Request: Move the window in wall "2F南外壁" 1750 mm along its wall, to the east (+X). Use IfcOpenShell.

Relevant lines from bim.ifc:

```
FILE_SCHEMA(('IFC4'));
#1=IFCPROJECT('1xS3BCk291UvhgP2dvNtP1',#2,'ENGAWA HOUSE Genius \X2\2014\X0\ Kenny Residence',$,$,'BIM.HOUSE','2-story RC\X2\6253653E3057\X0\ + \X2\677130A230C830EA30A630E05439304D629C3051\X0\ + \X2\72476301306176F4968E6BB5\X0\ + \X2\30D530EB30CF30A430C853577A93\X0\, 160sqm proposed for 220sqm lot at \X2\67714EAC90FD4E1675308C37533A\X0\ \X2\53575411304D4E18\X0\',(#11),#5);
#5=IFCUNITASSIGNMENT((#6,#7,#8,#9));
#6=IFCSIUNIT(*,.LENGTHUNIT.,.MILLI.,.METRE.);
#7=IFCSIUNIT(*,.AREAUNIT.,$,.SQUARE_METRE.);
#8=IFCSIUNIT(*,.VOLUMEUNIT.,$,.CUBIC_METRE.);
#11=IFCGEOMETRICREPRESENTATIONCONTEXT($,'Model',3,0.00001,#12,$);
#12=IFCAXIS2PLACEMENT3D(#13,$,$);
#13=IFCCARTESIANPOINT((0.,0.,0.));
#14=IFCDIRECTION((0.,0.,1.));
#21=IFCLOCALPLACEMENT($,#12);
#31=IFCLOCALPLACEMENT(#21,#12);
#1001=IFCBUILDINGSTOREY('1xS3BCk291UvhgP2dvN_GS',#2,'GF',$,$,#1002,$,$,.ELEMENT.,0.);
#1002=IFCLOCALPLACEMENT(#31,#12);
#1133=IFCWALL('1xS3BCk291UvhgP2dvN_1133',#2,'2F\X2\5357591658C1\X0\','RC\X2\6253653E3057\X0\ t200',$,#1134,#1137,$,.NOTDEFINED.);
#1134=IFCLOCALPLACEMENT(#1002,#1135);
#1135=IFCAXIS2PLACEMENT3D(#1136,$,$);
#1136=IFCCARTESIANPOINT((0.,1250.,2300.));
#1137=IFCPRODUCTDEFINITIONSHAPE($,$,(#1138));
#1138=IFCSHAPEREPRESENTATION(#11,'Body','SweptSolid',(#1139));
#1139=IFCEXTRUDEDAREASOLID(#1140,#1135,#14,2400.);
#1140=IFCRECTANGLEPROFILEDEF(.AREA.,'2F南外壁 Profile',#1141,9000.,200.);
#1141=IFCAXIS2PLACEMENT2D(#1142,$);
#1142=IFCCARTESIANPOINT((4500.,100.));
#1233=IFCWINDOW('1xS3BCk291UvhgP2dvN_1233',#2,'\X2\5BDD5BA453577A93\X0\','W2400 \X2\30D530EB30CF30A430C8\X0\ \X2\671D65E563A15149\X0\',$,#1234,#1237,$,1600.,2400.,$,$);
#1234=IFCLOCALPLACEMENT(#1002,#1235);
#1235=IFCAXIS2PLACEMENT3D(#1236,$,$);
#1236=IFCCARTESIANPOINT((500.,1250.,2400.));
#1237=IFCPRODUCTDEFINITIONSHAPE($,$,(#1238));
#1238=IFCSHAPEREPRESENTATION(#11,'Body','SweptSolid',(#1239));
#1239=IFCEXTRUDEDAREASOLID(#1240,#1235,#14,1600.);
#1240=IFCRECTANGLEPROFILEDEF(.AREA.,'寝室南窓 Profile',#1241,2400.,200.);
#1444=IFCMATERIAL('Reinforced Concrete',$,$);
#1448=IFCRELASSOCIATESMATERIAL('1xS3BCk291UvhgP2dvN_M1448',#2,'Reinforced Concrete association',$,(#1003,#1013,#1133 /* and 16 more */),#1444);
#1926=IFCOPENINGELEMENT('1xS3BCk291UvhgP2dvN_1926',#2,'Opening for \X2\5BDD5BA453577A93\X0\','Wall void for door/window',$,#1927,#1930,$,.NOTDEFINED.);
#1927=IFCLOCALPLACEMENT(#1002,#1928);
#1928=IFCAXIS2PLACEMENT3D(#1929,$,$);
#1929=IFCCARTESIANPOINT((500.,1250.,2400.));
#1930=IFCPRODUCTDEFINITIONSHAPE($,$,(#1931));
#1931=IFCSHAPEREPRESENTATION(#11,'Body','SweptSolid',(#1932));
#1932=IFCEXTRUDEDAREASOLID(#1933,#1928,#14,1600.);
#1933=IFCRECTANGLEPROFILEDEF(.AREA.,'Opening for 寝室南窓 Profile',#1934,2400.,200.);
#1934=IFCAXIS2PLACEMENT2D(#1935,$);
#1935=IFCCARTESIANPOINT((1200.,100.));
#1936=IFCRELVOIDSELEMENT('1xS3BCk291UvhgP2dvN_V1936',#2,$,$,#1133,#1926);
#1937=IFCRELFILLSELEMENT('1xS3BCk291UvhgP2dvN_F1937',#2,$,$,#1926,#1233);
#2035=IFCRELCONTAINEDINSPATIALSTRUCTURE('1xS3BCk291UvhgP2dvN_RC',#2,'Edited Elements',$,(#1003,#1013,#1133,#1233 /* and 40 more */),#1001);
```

```python
import ifcopenshell
import ifcopenshell.api.geometry
import ifcopenshell.util.placement
import ifcopenshell.util.unit

model = ifcopenshell.open("bim.ifc")
unit_scale = ifcopenshell.util.unit.calculate_unit_scale(model)

window = model.by_guid("1xS3BCk291UvhgP2dvN_1233")
opening = window.FillsVoids[0].RelatingOpeningElement
wall = opening.VoidsElements[0].RelatingBuildingElement

wall_matrix = ifcopenshell.util.placement.get_local_placement(wall.ObjectPlacement)
shift = wall_matrix[:3, 0] * 1.75 / unit_scale
before = ifcopenshell.util.placement.get_local_placement(window.ObjectPlacement)[:3, 3].copy()

# The window is not placed relative to its opening, so move both.
for product in (opening, window):
    matrix = ifcopenshell.util.placement.get_local_placement(product.ObjectPlacement)
    matrix[:3, 3] += shift
    ifcopenshell.api.geometry.edit_object_placement(model, product=product, matrix=matrix, is_si=False)

after = ifcopenshell.util.placement.get_local_placement(window.ObjectPlacement)[:3, 3]
print("window moved by", (after - before).round(3) + 0.0)

model.write("bim_rev.ifc")
```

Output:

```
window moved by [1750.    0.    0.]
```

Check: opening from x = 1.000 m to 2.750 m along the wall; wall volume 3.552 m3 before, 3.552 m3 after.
